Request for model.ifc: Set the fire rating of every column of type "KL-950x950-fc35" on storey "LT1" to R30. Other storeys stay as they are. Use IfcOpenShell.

First a look at what the model holds.

```python
import ifcopenshell
import ifcopenshell.util.element

model = ifcopenshell.open("model.ifc")
print(model.schema)
storey = next(s for s in model.by_type("IfcBuildingStorey") if s.Name == "LT1")
columns = [e for e in ifcopenshell.util.element.get_decomposition(storey) if e.is_a("IfcColumn")]
seen = {}
for e in columns:
    element_type = ifcopenshell.util.element.get_type(e)
    key = (element_type.Name if element_type != e and element_type else None, ifcopenshell.util.element.get_pset(e, "Pset_ColumnCommon", "FireRating"))
    seen[key] = seen.get(key, 0) + 1
for (name, value), count in sorted(seen.items(), key=str):
    print(count, "x", name, "|", value)
```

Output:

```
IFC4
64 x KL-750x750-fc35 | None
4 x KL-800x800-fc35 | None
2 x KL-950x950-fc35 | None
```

```python
import ifcopenshell
import ifcopenshell.api.pset
import ifcopenshell.util.element

model = ifcopenshell.open("model.ifc")

storey = next(s for s in model.by_type("IfcBuildingStorey") if s.Name == "LT1")
columns = [e for e in ifcopenshell.util.element.get_decomposition(storey) if e.is_a("IfcColumn")]

count = 0
for e in columns:
    element_type = ifcopenshell.util.element.get_type(e)
    if element_type in (None, e) or element_type.Name != "KL-950x950-fc35":
        continue
    # add_pset returns the element's existing set when there is one.
    pset = ifcopenshell.api.pset.add_pset(model, product=e, name="Pset_ColumnCommon")
    ifcopenshell.api.pset.edit_pset(model, pset=pset, properties={"FireRating": "R30"})
    count += 1

print(count, "columns updated")

model.write("model_rev.ifc")
```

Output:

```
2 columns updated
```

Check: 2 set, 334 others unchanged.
